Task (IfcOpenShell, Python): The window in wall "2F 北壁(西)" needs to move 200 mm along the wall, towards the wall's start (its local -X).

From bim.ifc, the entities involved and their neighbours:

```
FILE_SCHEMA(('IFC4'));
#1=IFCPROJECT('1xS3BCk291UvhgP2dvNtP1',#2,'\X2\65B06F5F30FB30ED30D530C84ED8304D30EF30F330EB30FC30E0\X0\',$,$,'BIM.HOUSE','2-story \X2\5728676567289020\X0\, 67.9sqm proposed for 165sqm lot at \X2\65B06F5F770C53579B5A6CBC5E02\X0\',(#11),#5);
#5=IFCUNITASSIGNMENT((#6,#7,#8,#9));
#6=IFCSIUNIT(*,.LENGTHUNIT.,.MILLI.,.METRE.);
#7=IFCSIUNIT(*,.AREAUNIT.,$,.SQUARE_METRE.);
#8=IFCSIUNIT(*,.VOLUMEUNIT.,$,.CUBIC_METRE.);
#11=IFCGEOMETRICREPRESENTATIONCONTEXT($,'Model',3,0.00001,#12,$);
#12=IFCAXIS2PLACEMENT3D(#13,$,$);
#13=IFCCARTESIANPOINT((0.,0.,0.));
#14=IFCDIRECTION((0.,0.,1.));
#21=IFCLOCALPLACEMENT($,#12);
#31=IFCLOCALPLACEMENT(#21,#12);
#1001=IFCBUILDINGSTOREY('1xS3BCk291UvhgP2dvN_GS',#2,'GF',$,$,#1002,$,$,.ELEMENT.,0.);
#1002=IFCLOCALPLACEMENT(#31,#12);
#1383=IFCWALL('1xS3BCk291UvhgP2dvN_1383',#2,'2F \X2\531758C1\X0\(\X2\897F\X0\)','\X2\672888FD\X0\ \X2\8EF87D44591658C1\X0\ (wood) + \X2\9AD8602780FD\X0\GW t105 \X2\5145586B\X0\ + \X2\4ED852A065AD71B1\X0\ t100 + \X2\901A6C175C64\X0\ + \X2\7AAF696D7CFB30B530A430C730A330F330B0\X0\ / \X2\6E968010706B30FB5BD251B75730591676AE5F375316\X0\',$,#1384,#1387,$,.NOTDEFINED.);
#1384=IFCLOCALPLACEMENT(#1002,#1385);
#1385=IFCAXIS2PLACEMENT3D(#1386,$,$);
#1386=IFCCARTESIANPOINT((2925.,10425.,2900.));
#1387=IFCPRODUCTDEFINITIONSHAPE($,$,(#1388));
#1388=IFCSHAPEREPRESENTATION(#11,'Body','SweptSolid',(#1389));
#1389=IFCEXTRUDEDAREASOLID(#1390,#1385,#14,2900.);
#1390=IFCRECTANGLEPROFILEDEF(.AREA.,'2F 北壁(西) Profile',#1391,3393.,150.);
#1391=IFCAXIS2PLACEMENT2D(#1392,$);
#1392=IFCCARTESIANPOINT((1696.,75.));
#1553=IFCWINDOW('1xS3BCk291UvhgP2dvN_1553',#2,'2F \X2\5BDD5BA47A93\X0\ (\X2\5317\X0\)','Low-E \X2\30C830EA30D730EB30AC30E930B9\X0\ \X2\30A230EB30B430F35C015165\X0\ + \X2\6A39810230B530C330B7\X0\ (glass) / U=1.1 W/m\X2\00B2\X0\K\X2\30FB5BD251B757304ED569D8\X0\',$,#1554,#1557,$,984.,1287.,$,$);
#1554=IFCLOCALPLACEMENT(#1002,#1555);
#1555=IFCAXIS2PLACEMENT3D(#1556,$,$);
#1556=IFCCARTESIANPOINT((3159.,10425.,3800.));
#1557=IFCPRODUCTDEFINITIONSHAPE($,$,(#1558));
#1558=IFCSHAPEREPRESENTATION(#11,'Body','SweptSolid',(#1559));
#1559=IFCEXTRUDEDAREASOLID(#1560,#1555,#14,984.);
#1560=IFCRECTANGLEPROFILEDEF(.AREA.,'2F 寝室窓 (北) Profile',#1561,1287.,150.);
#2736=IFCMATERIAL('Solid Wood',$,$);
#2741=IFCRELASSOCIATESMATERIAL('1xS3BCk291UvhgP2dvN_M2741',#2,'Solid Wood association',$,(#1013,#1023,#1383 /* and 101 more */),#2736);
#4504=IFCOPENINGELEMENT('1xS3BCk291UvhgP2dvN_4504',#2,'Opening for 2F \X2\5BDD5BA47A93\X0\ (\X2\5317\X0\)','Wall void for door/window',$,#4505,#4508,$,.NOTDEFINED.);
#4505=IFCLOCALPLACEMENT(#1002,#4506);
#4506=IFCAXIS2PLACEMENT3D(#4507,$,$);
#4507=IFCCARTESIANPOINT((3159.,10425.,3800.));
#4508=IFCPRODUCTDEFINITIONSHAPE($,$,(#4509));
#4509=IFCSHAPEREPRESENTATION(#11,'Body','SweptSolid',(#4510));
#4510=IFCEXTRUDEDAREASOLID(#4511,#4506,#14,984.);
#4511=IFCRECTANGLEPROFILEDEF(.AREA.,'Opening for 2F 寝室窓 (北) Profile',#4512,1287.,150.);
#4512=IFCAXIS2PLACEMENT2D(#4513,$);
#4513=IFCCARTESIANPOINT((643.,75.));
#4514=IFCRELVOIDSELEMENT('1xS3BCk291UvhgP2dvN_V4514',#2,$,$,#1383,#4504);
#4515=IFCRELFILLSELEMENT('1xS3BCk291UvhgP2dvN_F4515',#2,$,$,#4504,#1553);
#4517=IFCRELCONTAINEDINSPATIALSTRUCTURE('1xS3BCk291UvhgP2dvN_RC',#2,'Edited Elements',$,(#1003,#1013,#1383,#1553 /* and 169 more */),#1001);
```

```python
import ifcopenshell
import ifcopenshell.api.geometry
import ifcopenshell.util.placement
import ifcopenshell.util.unit

model = ifcopenshell.open("bim.ifc")
unit_scale = ifcopenshell.util.unit.calculate_unit_scale(model)

window = model.by_guid("1xS3BCk291UvhgP2dvN_1553")
opening = window.FillsVoids[0].RelatingOpeningElement
wall = opening.VoidsElements[0].RelatingBuildingElement

wall_matrix = ifcopenshell.util.placement.get_local_placement(wall.ObjectPlacement)
shift = wall_matrix[:3, 0] * -0.2 / unit_scale
before = ifcopenshell.util.placement.get_local_placement(window.ObjectPlacement)[:3, 3].copy()

# The window is not placed relative to its opening, so move both.
for product in (opening, window):
    matrix = ifcopenshell.util.placement.get_local_placement(product.ObjectPlacement)
    matrix[:3, 3] += shift
    ifcopenshell.api.geometry.edit_object_placement(model, product=product, matrix=matrix, is_si=False)

after = ifcopenshell.util.placement.get_local_placement(window.ObjectPlacement)[:3, 3]
print("window moved by", (after - before).round(3) + 0.0)

model.write("bim_v2.ifc")
```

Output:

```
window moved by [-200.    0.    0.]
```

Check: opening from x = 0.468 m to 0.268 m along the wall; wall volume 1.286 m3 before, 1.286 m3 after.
